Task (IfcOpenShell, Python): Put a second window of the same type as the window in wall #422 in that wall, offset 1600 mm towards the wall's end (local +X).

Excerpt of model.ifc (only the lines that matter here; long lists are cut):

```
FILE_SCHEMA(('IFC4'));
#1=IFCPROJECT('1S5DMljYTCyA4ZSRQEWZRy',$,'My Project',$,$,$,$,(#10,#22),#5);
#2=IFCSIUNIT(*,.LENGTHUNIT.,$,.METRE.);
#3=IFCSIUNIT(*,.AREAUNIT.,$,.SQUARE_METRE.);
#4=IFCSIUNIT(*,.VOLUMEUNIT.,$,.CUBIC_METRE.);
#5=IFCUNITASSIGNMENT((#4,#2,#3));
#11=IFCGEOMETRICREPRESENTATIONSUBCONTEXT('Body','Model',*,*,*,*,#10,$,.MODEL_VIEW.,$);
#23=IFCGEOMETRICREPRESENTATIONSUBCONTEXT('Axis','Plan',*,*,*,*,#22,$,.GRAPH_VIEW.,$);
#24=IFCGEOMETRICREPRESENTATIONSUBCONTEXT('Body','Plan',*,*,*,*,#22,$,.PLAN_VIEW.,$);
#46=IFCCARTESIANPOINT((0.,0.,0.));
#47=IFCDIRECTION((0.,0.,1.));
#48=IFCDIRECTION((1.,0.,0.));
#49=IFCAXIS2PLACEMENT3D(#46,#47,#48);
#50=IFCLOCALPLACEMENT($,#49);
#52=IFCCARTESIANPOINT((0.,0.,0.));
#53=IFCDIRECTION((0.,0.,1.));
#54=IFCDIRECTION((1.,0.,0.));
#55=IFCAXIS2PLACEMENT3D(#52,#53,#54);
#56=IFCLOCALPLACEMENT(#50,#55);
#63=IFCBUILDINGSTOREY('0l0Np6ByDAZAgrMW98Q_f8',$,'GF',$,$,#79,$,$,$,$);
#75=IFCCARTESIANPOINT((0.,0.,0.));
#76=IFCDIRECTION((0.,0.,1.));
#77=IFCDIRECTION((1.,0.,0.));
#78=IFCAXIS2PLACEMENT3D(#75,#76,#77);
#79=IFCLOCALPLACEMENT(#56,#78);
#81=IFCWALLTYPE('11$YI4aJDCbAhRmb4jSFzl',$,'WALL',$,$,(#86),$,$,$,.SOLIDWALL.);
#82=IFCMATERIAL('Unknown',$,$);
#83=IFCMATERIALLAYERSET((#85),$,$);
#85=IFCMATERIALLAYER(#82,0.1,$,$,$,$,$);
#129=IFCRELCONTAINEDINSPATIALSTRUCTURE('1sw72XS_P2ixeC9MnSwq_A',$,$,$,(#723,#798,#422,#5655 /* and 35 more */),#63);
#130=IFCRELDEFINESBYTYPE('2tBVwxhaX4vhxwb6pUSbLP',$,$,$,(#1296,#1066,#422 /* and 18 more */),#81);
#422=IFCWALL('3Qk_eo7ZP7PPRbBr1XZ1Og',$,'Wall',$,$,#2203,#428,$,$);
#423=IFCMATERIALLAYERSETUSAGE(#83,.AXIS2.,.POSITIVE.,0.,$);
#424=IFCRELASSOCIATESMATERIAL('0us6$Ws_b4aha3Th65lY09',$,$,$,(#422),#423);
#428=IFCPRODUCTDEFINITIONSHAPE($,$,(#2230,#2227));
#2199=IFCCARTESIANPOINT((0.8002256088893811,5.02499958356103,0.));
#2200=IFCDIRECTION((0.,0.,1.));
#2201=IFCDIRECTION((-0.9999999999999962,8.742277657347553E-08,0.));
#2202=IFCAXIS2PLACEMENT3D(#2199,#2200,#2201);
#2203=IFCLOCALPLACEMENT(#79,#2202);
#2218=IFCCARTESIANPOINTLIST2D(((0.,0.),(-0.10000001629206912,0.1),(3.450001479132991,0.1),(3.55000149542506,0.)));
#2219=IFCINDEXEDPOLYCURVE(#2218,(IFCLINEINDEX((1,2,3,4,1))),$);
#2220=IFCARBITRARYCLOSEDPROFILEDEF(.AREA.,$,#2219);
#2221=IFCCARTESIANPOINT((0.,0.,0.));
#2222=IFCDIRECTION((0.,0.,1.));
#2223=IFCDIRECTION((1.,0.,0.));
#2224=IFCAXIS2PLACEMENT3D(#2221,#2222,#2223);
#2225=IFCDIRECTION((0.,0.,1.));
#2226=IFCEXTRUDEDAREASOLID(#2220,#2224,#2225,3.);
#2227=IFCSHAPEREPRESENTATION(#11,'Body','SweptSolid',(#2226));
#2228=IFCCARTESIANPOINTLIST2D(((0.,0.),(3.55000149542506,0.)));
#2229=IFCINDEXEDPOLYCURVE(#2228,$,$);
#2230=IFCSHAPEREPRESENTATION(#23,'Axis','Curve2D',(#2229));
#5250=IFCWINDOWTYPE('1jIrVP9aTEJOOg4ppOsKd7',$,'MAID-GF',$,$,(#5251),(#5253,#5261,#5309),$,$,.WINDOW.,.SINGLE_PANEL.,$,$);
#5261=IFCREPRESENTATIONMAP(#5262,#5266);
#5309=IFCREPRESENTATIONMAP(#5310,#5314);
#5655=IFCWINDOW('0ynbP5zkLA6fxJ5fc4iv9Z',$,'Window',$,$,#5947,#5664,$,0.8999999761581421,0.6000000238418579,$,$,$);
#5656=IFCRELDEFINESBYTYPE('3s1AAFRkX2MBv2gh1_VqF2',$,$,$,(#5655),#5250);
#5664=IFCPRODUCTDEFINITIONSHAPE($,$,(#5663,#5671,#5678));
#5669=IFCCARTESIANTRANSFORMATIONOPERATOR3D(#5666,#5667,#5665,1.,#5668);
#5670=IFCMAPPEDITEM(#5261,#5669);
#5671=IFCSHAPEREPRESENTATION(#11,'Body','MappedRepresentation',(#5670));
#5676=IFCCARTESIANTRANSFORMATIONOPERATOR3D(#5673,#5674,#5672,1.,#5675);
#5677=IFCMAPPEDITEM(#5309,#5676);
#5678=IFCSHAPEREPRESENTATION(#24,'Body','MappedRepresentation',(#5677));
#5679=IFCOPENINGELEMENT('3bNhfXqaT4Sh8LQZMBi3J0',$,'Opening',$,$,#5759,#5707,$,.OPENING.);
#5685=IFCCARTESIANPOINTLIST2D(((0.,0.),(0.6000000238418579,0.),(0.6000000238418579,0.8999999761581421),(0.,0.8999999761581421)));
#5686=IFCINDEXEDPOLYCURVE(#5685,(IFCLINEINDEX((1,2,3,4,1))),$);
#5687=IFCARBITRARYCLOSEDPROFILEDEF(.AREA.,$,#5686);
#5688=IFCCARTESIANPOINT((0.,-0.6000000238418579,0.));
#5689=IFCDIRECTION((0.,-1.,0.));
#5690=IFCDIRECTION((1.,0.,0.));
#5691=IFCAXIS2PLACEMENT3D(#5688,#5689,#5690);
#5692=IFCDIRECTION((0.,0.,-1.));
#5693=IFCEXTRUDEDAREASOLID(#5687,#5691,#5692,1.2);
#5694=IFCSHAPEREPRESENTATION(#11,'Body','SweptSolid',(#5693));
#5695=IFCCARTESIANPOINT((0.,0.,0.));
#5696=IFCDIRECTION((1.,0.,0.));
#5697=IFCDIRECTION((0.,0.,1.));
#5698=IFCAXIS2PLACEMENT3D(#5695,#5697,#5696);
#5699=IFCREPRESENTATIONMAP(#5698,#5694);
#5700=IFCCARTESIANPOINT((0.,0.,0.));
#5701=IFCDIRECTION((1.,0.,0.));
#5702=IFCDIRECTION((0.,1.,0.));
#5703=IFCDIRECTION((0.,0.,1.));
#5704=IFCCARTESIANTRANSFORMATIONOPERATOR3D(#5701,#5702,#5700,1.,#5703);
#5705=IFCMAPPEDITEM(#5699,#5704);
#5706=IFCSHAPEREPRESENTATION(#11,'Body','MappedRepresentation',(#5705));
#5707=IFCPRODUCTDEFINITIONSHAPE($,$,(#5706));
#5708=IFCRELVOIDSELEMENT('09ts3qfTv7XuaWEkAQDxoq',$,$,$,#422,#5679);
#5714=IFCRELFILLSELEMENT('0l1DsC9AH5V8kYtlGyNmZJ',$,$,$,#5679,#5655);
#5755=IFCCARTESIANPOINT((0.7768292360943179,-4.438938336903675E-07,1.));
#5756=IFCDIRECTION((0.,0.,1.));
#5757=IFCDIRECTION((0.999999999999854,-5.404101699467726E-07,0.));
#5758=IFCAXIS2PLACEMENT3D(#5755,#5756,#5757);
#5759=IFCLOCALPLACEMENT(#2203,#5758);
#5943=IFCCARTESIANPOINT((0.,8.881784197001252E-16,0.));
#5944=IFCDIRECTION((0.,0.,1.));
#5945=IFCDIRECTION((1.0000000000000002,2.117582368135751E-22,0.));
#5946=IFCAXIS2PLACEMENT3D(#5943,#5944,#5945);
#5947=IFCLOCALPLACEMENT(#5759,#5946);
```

```python
import ifcopenshell
import ifcopenshell.api.feature
import ifcopenshell.api.geometry
import ifcopenshell.api.root
import ifcopenshell.geom
import ifcopenshell.util.element
import ifcopenshell.util.placement
import ifcopenshell.util.shape
import ifcopenshell.util.unit

model = ifcopenshell.open("model.ifc")
unit_scale = ifcopenshell.util.unit.calculate_unit_scale(model)
settings = ifcopenshell.geom.settings()


def volume(element):
    """Net volume in cubic metres, openings subtracted."""
    shape = ifcopenshell.geom.create_shape(settings, element)
    return ifcopenshell.util.shape.get_volume(shape.geometry)


window = model.by_id(5655)
opening = window.FillsVoids[0].RelatingOpeningElement
wall = opening.VoidsElements[0].RelatingBuildingElement
before = volume(wall)
shift = ifcopenshell.util.placement.get_local_placement(wall.ObjectPlacement)[:3, 0] * 1.6 / unit_scale

# copy_class copies the void relationship, type, container and properties, but no geometry.
new_opening = ifcopenshell.api.root.copy_class(model, product=opening)
new_opening.Representation = ifcopenshell.util.element.copy_deep(
    model, opening.Representation, exclude=["IfcGeometricRepresentationContext", "IfcRepresentationMap"]
)
new_window = ifcopenshell.api.root.copy_class(model, product=window)
new_window.Representation = ifcopenshell.util.element.copy_deep(
    model, window.Representation, exclude=["IfcGeometricRepresentationContext", "IfcRepresentationMap"]
)
ifcopenshell.api.feature.add_filling(model, opening=new_opening, element=new_window)

for old, new in ((opening, new_opening), (window, new_window)):
    matrix = ifcopenshell.util.placement.get_local_placement(old.ObjectPlacement)
    matrix[:3, 3] += shift
    ifcopenshell.api.geometry.edit_object_placement(model, product=new, matrix=matrix, is_si=False)

after = volume(wall)

print(f"wall volume {before:.3f} -> {after:.3f} m3")

model.write("model_rev.ifc")
```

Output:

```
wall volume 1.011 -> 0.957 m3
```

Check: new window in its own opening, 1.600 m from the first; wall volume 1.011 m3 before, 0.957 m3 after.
